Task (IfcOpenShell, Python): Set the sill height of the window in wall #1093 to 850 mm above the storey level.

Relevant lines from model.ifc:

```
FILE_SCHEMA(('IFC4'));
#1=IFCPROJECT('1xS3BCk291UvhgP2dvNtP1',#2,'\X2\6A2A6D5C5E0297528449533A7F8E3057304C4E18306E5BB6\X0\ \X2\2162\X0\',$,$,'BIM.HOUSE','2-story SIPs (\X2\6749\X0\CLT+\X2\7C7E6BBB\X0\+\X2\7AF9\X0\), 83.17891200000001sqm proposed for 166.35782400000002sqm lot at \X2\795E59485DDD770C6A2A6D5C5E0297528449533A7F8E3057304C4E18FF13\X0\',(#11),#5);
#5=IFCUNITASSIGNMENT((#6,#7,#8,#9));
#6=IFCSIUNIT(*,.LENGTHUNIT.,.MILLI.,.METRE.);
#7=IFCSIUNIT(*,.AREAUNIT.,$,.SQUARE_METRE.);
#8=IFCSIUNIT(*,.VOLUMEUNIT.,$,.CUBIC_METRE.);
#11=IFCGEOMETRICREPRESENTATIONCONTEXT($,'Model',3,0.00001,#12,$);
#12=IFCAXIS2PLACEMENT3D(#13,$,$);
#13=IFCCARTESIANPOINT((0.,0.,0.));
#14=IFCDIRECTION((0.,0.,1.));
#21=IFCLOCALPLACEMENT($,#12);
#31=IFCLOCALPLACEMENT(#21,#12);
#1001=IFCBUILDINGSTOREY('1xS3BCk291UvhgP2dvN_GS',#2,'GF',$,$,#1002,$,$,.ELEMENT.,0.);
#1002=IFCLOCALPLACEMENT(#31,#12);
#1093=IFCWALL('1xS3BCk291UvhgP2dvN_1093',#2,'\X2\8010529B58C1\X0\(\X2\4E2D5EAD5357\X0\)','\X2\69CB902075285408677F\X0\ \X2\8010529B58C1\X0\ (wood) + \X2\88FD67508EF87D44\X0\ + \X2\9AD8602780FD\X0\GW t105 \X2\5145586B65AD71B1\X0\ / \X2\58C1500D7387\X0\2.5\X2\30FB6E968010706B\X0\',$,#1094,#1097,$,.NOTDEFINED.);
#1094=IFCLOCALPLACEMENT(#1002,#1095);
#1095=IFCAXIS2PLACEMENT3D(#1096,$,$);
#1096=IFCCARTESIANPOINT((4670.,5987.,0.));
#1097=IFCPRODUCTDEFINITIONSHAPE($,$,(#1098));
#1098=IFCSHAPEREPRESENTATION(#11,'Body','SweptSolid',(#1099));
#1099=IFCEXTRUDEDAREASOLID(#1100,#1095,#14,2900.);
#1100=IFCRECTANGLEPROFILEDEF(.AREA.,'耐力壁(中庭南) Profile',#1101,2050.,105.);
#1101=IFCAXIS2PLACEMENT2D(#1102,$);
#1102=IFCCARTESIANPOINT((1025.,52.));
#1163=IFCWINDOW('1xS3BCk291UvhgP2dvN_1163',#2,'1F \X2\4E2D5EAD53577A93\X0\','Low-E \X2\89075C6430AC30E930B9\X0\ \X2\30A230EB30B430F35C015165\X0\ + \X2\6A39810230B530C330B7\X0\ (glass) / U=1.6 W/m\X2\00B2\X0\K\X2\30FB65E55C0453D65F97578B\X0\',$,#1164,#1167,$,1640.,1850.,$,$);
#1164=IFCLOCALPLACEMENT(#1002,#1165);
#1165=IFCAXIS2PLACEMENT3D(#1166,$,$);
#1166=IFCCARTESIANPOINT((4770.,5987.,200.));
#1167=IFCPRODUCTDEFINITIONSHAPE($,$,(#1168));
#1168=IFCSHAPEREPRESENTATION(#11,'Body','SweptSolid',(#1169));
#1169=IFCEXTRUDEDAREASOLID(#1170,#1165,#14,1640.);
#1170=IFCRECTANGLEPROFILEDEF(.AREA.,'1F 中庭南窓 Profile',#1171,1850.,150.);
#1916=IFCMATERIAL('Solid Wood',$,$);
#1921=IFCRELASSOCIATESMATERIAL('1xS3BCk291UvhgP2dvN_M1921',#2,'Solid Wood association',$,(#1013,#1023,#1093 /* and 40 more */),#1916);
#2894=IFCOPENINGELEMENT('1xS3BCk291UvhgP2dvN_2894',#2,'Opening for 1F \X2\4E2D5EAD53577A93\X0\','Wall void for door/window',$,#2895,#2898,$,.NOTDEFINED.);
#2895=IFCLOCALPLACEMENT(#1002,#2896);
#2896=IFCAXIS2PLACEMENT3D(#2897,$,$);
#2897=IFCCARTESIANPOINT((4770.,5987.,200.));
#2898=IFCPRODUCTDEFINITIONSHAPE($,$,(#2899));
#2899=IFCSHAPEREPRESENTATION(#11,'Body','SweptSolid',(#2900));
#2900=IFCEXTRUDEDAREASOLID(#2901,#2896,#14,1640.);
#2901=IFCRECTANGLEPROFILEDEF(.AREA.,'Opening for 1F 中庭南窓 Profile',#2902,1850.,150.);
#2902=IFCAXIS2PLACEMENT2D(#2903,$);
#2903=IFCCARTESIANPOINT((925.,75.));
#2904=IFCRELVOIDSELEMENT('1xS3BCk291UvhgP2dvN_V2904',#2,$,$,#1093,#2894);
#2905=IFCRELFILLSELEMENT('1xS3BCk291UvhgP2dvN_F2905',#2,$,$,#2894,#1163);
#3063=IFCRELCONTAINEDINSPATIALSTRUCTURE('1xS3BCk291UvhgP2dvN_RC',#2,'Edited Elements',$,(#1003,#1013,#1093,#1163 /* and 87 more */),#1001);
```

```python
import numpy as np
import ifcopenshell
import ifcopenshell.api.geometry
import ifcopenshell.geom
import ifcopenshell.util.element
import ifcopenshell.util.placement
import ifcopenshell.util.shape
import ifcopenshell.util.unit

model = ifcopenshell.open("model.ifc")
unit_scale = ifcopenshell.util.unit.calculate_unit_scale(model)

window = model.by_guid("1xS3BCk291UvhgP2dvN_1163")
opening = window.FillsVoids[0].RelatingOpeningElement
storey = ifcopenshell.util.element.get_container(window, ifc_class="IfcBuildingStorey")
level = ifcopenshell.util.placement.get_local_placement(storey.ObjectPlacement)[2, 3]

# The opening's origin need not be at the sill, so measure its lowest point.
shape = ifcopenshell.geom.create_shape(ifcopenshell.geom.settings(), opening)
bottom = ifcopenshell.util.shape.get_shape_bottom_elevation(shape, shape.geometry) / unit_scale
dz = level + 0.85 / unit_scale - bottom

shift = np.array([0.0, 0.0, dz])
# The window is not placed relative to its opening, so move both.
for product in (opening, window):
    matrix = ifcopenshell.util.placement.get_local_placement(product.ObjectPlacement)
    matrix[:3, 3] += shift
    ifcopenshell.api.geometry.edit_object_placement(model, product=product, matrix=matrix, is_si=False)

print(f"moved by {dz * unit_scale:+.3f} m")

model.write("model_v2.ifc")
```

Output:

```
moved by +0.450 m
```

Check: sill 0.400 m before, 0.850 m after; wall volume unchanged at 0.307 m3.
